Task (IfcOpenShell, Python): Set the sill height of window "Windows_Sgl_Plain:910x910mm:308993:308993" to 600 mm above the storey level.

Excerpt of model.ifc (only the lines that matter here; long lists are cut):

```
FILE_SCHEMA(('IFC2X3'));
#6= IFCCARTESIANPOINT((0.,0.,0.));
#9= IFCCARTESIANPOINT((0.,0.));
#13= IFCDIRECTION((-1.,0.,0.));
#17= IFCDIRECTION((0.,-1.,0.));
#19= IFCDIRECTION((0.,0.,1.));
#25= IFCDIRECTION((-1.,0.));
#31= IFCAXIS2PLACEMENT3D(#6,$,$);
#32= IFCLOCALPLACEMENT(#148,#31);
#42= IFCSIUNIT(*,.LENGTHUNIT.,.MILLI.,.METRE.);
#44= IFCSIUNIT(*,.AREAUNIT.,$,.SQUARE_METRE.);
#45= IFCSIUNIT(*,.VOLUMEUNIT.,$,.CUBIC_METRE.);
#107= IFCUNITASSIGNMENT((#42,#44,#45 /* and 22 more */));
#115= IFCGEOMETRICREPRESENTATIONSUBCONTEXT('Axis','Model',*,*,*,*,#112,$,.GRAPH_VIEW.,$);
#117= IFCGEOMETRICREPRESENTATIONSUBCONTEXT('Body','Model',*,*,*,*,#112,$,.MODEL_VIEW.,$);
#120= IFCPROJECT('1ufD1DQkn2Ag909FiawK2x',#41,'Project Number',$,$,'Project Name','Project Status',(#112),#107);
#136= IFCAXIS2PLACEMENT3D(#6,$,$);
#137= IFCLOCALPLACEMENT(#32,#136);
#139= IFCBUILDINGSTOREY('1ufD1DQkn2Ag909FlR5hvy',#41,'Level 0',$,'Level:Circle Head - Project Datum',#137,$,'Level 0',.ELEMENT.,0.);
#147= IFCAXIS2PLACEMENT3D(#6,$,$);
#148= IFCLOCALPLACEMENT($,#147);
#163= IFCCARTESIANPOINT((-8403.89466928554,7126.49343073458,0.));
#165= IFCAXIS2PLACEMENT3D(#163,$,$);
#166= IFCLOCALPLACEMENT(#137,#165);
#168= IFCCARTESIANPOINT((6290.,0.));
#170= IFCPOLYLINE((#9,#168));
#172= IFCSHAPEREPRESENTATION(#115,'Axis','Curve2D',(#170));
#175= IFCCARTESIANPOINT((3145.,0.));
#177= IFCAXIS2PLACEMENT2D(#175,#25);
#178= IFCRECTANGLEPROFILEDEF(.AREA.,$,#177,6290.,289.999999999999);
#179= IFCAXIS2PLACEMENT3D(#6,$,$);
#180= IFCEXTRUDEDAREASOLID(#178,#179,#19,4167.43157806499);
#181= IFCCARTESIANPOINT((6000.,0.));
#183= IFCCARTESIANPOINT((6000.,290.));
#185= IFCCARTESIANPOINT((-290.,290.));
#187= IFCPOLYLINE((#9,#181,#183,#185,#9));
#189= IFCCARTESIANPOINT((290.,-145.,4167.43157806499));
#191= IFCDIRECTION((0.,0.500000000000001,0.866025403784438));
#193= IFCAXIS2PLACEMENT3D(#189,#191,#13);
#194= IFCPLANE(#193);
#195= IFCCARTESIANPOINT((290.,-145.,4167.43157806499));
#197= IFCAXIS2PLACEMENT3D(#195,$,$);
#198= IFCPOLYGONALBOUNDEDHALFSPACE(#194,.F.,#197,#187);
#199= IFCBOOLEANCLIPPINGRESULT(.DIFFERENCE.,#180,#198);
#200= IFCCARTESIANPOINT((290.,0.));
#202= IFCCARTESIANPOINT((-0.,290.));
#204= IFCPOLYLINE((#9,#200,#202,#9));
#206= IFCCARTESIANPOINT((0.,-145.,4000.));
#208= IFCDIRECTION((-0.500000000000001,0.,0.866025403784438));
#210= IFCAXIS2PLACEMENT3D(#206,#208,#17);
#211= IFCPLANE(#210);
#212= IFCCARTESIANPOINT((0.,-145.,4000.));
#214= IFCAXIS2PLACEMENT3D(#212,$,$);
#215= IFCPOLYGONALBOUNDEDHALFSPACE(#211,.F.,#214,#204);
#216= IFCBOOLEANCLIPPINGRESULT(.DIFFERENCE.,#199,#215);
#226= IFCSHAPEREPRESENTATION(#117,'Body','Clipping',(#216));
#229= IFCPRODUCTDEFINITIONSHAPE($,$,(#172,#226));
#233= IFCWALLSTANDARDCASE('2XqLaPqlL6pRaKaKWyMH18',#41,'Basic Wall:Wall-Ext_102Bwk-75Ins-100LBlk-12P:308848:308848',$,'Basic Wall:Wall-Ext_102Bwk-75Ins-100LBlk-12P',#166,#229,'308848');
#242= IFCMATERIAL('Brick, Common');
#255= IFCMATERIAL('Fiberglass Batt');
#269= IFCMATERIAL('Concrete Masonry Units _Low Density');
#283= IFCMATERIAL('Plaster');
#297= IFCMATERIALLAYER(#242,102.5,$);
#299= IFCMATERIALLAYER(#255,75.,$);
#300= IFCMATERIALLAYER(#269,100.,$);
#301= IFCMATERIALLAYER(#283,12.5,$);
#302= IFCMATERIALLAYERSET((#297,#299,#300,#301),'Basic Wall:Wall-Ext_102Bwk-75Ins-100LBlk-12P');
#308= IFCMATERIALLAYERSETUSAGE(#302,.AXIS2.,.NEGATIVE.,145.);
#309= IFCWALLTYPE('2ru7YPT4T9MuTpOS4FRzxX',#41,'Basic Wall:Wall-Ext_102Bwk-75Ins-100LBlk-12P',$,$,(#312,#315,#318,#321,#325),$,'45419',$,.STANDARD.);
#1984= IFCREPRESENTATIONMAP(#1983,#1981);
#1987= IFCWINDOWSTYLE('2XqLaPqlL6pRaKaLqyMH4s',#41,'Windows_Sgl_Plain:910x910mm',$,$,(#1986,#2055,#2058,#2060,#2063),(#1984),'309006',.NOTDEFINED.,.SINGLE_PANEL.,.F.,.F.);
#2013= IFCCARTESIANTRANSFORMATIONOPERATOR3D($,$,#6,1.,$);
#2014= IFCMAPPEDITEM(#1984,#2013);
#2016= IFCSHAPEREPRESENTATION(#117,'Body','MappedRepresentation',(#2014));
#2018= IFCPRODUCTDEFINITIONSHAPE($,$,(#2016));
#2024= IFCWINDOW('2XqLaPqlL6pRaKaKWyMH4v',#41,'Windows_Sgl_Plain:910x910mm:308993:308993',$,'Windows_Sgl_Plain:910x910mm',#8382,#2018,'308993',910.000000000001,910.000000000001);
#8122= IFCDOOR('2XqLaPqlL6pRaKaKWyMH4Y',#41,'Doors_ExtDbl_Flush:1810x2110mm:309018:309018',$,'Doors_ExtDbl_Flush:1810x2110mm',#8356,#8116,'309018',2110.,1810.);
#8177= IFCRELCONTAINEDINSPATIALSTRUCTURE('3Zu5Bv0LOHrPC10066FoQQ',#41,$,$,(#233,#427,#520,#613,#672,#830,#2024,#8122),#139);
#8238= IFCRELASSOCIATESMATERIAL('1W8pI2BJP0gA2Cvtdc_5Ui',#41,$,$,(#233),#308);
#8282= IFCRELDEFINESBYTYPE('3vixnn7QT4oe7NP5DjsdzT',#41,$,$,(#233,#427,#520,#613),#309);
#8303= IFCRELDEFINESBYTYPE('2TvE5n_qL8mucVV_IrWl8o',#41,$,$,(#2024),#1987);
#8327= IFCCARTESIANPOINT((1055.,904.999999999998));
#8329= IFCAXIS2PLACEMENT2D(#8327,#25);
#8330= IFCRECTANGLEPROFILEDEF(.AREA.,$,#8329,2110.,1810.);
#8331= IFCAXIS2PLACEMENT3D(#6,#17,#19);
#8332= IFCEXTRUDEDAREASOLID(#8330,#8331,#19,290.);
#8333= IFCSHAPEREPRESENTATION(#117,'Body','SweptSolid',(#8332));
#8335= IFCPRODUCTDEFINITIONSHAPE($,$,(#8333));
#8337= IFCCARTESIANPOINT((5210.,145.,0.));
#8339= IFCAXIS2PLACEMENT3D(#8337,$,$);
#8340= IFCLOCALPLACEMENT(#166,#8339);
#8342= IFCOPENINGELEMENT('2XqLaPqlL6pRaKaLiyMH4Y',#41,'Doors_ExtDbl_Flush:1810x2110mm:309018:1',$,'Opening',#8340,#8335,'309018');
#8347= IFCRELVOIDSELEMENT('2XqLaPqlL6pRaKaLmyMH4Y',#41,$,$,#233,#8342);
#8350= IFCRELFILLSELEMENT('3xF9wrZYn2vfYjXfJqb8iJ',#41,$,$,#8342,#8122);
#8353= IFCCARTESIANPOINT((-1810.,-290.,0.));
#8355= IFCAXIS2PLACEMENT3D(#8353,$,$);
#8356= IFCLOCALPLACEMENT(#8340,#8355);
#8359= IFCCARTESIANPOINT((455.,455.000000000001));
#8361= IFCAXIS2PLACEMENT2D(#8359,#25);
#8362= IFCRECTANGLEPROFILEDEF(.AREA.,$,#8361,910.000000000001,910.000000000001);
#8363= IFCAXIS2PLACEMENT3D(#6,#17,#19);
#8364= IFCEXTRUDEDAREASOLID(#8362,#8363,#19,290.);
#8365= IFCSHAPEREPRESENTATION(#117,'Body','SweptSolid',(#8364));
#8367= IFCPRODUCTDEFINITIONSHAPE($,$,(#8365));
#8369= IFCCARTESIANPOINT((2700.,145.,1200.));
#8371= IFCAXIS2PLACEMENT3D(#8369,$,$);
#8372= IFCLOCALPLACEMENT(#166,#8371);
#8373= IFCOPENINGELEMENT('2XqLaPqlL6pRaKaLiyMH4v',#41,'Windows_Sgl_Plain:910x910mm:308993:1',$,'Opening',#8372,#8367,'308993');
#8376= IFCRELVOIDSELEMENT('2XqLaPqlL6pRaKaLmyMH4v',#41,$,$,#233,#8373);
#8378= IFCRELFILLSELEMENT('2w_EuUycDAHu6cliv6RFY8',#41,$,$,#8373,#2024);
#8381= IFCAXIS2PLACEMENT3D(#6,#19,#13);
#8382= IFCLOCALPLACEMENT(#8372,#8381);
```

```python
import numpy as np
import ifcopenshell
import ifcopenshell.api.geometry
import ifcopenshell.geom
import ifcopenshell.util.element
import ifcopenshell.util.placement
import ifcopenshell.util.shape
import ifcopenshell.util.unit

model = ifcopenshell.open("model.ifc")
unit_scale = ifcopenshell.util.unit.calculate_unit_scale(model)

window = model.by_id(2024)
opening = window.FillsVoids[0].RelatingOpeningElement
storey = ifcopenshell.util.element.get_container(window, ifc_class="IfcBuildingStorey")
level = ifcopenshell.util.placement.get_local_placement(storey.ObjectPlacement)[2, 3]

# The opening's origin need not be at the sill, so measure its lowest point.
shape = ifcopenshell.geom.create_shape(ifcopenshell.geom.settings(), opening)
bottom = ifcopenshell.util.shape.get_shape_bottom_elevation(shape, shape.geometry) / unit_scale
dz = level + 0.6 / unit_scale - bottom

shift = np.array([0.0, 0.0, dz])
# The window is placed relative to its opening, so it follows when the opening moves.
matrix = ifcopenshell.util.placement.get_local_placement(opening.ObjectPlacement)
matrix[:3, 3] += shift
ifcopenshell.api.geometry.edit_object_placement(
    model, product=opening, matrix=matrix, is_si=False, should_transform_children=True
)

print(f"moved by {dz * unit_scale:+.3f} m")

model.write("model_rev.ifc")
```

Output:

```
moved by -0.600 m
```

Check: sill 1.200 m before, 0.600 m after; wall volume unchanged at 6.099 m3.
